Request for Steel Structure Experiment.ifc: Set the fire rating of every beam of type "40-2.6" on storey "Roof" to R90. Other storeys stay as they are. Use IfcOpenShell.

First a look at what the model holds.

```python
import ifcopenshell
import ifcopenshell.util.element

model = ifcopenshell.open("Steel Structure Experiment.ifc")
print(model.schema)
storey = next(s for s in model.by_type("IfcBuildingStorey") if s.Name == "Roof")
beams = [e for e in ifcopenshell.util.element.get_decomposition(storey) if e.is_a("IfcBeam")]
seen = {}
for e in beams:
    element_type = ifcopenshell.util.element.get_type(e)
    key = (element_type.Name if element_type != e and element_type else None, ifcopenshell.util.element.get_pset(e, "Pset_BeamCommon", "FireRating"))
    seen[key] = seen.get(key, 0) + 1
for (name, value), count in sorted(seen.items(), key=str):
    print(count, "x", name, "|", value)
```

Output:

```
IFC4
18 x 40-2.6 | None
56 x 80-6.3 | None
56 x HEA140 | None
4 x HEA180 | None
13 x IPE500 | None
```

```python
import ifcopenshell
import ifcopenshell.api.pset
import ifcopenshell.util.element

model = ifcopenshell.open("Steel Structure Experiment.ifc")

storey = next(s for s in model.by_type("IfcBuildingStorey") if s.Name == "Roof")
beams = [e for e in ifcopenshell.util.element.get_decomposition(storey) if e.is_a("IfcBeam")]

count = 0
for e in beams:
    element_type = ifcopenshell.util.element.get_type(e)
    if element_type in (None, e) or element_type.Name != "40-2.6":
        continue
    # add_pset returns the element's existing set when there is one.
    pset = ifcopenshell.api.pset.add_pset(model, product=e, name="Pset_BeamCommon")
    ifcopenshell.api.pset.edit_pset(model, pset=pset, properties={"FireRating": "R90"})
    count += 1

print(count, "beams updated")

model.write("Steel Structure Experiment_updated.ifc")
```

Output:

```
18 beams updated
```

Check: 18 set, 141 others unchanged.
